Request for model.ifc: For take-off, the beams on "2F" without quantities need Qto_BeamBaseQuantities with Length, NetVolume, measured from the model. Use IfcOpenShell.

First a look at what the model holds.

```python
import ifcopenshell
import ifcopenshell.util.element
import ifcopenshell.util.unit

model = ifcopenshell.open("model.ifc")
print(model.schema)
for unit_type in ("LENGTHUNIT", "AREAUNIT", "VOLUMEUNIT"):
    print(unit_type, ifcopenshell.util.unit.calculate_unit_scale(model, unit_type))
storey = next(s for s in model.by_type("IfcBuildingStorey") if s.Name == "2F")
beams = [e for e in ifcopenshell.util.element.get_decomposition(storey) if e.is_a("IfcBeam")]
for e in sorted(beams, key=lambda e: e.id()):
    print(e.id(), e.is_a(), e.Name, list(ifcopenshell.util.element.get_psets(e, qtos_only=True)), sep=" | ")
```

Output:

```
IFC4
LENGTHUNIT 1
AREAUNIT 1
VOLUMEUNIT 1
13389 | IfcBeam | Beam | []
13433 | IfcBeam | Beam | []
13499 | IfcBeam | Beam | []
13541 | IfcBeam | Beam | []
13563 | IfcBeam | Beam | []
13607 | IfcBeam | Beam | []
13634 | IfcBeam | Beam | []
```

```python
import ifcopenshell
import ifcopenshell.api.pset
import ifcopenshell.geom
import ifcopenshell.util.element
import ifcopenshell.util.shape
import ifcopenshell.util.unit

model = ifcopenshell.open("model.ifc")
unit_scale = ifcopenshell.util.unit.calculate_unit_scale(model)
volume_scale = ifcopenshell.util.unit.calculate_unit_scale(model, "VOLUMEUNIT")
settings = ifcopenshell.geom.settings()

storey = next(s for s in model.by_type("IfcBuildingStorey") if s.Name == "2F")
beams = [e for e in ifcopenshell.util.element.get_decomposition(storey) if e.is_a("IfcBeam")]

for e in sorted(beams, key=lambda e: e.id()):
    if ifcopenshell.util.element.get_psets(e, qtos_only=True, should_inherit=False):
        continue
    # Geometry comes back in metres, in the element's own axes.
    shape = ifcopenshell.geom.create_shape(settings, e)
    values = {
        "Length": ifcopenshell.util.shape.get_max_xyz(shape.geometry) / unit_scale,
        "NetVolume": ifcopenshell.util.shape.get_volume(shape.geometry) / volume_scale,
    }
    qto = ifcopenshell.api.pset.add_qto(model, product=e, name="Qto_BeamBaseQuantities")
    ifcopenshell.api.pset.edit_qto(model, qto=qto, properties=values)
    print(e.id(), {k: round(v, 3) for k, v in values.items()})

model.write("model_v2.ifc")
```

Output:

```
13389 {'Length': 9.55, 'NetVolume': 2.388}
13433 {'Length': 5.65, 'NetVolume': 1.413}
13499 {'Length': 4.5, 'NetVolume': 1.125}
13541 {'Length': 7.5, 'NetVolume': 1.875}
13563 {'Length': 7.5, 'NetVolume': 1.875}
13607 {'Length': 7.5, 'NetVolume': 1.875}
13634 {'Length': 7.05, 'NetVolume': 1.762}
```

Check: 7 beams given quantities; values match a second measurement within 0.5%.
